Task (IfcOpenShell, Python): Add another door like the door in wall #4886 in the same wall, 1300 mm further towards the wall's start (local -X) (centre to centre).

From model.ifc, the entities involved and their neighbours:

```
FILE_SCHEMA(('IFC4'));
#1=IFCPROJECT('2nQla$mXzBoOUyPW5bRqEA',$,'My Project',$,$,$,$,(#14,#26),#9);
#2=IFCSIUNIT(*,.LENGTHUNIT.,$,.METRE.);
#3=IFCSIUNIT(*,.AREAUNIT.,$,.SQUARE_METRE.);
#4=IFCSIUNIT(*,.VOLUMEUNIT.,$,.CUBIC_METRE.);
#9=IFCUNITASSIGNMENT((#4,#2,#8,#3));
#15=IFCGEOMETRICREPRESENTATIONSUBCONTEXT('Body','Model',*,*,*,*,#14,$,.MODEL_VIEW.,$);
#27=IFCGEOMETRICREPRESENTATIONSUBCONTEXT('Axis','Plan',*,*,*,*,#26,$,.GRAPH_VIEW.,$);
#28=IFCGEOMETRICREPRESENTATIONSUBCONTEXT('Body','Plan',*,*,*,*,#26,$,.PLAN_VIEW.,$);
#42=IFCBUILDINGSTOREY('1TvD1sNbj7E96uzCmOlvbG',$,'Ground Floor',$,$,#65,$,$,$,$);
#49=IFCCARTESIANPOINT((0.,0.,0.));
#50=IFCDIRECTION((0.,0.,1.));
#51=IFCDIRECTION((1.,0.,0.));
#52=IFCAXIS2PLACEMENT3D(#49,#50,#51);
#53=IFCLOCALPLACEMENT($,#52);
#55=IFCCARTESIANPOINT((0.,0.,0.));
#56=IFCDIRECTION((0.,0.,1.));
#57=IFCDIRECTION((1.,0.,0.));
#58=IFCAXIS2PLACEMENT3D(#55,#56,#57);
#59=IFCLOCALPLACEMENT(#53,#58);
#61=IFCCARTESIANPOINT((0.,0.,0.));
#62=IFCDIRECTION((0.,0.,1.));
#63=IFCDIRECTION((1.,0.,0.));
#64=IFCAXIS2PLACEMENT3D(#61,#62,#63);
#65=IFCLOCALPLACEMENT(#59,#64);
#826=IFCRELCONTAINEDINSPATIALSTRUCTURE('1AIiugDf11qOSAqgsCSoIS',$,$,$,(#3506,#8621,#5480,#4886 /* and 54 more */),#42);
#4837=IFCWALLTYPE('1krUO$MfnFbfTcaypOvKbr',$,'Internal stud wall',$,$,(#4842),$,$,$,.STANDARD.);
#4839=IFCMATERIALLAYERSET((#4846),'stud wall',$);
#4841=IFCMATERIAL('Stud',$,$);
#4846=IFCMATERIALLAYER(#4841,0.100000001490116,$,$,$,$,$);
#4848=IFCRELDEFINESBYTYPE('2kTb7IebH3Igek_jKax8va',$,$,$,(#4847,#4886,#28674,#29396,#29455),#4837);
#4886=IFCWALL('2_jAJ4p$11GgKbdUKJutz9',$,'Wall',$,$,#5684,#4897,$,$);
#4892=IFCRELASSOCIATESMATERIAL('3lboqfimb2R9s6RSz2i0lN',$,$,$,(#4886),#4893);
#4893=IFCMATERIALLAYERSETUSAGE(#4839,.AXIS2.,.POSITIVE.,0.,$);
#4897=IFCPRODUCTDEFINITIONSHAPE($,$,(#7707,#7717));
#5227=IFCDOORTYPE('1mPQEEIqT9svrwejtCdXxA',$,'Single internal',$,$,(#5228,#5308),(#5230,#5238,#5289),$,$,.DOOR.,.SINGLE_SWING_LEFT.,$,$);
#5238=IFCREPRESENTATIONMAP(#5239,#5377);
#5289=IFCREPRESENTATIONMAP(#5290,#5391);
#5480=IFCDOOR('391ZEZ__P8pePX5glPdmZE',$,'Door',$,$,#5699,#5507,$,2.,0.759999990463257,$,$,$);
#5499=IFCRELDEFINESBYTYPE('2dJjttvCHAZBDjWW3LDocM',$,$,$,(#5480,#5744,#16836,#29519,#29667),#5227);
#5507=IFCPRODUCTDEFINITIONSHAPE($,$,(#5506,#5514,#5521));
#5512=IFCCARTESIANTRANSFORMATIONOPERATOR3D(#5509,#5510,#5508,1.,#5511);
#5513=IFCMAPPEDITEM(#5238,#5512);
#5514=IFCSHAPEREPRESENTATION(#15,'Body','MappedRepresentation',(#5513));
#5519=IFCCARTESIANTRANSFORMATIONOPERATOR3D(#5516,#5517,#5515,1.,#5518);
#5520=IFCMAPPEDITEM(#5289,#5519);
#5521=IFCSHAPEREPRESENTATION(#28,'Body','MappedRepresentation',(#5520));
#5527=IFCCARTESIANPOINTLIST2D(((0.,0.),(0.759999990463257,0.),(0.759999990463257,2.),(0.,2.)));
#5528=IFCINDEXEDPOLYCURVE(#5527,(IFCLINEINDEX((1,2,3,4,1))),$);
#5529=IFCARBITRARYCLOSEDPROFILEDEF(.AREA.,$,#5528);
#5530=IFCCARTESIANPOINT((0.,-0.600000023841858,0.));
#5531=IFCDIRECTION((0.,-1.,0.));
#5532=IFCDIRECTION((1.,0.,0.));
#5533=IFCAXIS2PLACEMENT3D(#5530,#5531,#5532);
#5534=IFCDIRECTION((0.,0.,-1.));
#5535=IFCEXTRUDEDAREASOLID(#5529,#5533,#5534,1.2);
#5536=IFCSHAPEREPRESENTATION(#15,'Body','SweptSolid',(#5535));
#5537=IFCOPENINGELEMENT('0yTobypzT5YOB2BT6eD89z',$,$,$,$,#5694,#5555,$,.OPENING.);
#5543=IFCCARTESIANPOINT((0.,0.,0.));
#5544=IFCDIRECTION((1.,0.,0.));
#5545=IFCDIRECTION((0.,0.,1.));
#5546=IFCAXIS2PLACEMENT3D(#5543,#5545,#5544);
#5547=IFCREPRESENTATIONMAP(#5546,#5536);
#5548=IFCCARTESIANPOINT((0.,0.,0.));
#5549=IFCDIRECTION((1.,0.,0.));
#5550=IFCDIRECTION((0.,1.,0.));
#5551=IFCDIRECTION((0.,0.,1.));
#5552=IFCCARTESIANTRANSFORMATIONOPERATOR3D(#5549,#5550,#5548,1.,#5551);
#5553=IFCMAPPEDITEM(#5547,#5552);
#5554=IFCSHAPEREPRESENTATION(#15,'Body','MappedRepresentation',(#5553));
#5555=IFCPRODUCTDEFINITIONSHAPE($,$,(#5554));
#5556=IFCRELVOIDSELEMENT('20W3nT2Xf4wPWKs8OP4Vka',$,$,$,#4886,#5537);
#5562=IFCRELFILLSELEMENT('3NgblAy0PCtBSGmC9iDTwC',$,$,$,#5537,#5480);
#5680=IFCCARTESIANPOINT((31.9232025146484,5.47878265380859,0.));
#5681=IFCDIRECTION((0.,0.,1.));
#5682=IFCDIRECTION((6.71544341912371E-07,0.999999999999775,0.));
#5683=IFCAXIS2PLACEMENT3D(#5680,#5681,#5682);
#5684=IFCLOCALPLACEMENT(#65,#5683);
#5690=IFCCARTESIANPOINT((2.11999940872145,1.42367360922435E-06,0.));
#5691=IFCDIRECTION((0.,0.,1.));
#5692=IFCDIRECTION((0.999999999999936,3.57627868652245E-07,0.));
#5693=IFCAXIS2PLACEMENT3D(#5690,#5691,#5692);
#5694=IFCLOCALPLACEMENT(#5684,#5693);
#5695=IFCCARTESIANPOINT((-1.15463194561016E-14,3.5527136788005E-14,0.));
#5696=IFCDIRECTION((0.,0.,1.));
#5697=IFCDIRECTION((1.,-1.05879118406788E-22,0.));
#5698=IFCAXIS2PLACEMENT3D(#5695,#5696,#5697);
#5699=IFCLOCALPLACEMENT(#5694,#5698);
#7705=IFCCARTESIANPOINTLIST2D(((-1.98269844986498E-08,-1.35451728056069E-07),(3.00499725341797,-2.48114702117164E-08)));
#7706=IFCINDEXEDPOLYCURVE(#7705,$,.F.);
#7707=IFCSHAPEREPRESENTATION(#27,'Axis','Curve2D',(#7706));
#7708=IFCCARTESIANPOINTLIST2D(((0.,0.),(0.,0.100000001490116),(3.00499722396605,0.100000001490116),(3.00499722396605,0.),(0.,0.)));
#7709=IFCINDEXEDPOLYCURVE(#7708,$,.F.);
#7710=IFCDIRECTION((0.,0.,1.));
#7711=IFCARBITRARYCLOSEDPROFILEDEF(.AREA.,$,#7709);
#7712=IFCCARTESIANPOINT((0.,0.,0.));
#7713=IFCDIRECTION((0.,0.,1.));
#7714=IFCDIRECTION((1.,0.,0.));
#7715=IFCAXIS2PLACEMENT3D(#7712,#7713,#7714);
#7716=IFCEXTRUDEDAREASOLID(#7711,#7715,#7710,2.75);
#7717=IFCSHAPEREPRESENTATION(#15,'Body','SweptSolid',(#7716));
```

```python
import ifcopenshell
import ifcopenshell.api.feature
import ifcopenshell.api.geometry
import ifcopenshell.api.root
import ifcopenshell.geom
import ifcopenshell.util.element
import ifcopenshell.util.placement
import ifcopenshell.util.shape
import ifcopenshell.util.unit

model = ifcopenshell.open("model.ifc")
unit_scale = ifcopenshell.util.unit.calculate_unit_scale(model)
settings = ifcopenshell.geom.settings()


def volume(element):
    """Net volume in cubic metres, openings subtracted."""
    shape = ifcopenshell.geom.create_shape(settings, element)
    return ifcopenshell.util.shape.get_volume(shape.geometry)


door = model.by_id(5480)
opening = door.FillsVoids[0].RelatingOpeningElement
wall = opening.VoidsElements[0].RelatingBuildingElement
before = volume(wall)
shift = ifcopenshell.util.placement.get_local_placement(wall.ObjectPlacement)[:3, 0] * -1.3 / unit_scale

# copy_class copies the void relationship, type, container and properties, but no geometry.
new_opening = ifcopenshell.api.root.copy_class(model, product=opening)
new_opening.Representation = ifcopenshell.util.element.copy_deep(
    model, opening.Representation, exclude=["IfcGeometricRepresentationContext", "IfcRepresentationMap"]
)
new_door = ifcopenshell.api.root.copy_class(model, product=door)
new_door.Representation = ifcopenshell.util.element.copy_deep(
    model, door.Representation, exclude=["IfcGeometricRepresentationContext", "IfcRepresentationMap"]
)
ifcopenshell.api.feature.add_filling(model, opening=new_opening, element=new_door)

for old, new in ((opening, new_opening), (door, new_door)):
    matrix = ifcopenshell.util.placement.get_local_placement(old.ObjectPlacement)
    matrix[:3, 3] += shift
    ifcopenshell.api.geometry.edit_object_placement(model, product=new, matrix=matrix, is_si=False)

after = volume(wall)

print(f"wall volume {before:.3f} -> {after:.3f} m3")

model.write("model-out.ifc")
```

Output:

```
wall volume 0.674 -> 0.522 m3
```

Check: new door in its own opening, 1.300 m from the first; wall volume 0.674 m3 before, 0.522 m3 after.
